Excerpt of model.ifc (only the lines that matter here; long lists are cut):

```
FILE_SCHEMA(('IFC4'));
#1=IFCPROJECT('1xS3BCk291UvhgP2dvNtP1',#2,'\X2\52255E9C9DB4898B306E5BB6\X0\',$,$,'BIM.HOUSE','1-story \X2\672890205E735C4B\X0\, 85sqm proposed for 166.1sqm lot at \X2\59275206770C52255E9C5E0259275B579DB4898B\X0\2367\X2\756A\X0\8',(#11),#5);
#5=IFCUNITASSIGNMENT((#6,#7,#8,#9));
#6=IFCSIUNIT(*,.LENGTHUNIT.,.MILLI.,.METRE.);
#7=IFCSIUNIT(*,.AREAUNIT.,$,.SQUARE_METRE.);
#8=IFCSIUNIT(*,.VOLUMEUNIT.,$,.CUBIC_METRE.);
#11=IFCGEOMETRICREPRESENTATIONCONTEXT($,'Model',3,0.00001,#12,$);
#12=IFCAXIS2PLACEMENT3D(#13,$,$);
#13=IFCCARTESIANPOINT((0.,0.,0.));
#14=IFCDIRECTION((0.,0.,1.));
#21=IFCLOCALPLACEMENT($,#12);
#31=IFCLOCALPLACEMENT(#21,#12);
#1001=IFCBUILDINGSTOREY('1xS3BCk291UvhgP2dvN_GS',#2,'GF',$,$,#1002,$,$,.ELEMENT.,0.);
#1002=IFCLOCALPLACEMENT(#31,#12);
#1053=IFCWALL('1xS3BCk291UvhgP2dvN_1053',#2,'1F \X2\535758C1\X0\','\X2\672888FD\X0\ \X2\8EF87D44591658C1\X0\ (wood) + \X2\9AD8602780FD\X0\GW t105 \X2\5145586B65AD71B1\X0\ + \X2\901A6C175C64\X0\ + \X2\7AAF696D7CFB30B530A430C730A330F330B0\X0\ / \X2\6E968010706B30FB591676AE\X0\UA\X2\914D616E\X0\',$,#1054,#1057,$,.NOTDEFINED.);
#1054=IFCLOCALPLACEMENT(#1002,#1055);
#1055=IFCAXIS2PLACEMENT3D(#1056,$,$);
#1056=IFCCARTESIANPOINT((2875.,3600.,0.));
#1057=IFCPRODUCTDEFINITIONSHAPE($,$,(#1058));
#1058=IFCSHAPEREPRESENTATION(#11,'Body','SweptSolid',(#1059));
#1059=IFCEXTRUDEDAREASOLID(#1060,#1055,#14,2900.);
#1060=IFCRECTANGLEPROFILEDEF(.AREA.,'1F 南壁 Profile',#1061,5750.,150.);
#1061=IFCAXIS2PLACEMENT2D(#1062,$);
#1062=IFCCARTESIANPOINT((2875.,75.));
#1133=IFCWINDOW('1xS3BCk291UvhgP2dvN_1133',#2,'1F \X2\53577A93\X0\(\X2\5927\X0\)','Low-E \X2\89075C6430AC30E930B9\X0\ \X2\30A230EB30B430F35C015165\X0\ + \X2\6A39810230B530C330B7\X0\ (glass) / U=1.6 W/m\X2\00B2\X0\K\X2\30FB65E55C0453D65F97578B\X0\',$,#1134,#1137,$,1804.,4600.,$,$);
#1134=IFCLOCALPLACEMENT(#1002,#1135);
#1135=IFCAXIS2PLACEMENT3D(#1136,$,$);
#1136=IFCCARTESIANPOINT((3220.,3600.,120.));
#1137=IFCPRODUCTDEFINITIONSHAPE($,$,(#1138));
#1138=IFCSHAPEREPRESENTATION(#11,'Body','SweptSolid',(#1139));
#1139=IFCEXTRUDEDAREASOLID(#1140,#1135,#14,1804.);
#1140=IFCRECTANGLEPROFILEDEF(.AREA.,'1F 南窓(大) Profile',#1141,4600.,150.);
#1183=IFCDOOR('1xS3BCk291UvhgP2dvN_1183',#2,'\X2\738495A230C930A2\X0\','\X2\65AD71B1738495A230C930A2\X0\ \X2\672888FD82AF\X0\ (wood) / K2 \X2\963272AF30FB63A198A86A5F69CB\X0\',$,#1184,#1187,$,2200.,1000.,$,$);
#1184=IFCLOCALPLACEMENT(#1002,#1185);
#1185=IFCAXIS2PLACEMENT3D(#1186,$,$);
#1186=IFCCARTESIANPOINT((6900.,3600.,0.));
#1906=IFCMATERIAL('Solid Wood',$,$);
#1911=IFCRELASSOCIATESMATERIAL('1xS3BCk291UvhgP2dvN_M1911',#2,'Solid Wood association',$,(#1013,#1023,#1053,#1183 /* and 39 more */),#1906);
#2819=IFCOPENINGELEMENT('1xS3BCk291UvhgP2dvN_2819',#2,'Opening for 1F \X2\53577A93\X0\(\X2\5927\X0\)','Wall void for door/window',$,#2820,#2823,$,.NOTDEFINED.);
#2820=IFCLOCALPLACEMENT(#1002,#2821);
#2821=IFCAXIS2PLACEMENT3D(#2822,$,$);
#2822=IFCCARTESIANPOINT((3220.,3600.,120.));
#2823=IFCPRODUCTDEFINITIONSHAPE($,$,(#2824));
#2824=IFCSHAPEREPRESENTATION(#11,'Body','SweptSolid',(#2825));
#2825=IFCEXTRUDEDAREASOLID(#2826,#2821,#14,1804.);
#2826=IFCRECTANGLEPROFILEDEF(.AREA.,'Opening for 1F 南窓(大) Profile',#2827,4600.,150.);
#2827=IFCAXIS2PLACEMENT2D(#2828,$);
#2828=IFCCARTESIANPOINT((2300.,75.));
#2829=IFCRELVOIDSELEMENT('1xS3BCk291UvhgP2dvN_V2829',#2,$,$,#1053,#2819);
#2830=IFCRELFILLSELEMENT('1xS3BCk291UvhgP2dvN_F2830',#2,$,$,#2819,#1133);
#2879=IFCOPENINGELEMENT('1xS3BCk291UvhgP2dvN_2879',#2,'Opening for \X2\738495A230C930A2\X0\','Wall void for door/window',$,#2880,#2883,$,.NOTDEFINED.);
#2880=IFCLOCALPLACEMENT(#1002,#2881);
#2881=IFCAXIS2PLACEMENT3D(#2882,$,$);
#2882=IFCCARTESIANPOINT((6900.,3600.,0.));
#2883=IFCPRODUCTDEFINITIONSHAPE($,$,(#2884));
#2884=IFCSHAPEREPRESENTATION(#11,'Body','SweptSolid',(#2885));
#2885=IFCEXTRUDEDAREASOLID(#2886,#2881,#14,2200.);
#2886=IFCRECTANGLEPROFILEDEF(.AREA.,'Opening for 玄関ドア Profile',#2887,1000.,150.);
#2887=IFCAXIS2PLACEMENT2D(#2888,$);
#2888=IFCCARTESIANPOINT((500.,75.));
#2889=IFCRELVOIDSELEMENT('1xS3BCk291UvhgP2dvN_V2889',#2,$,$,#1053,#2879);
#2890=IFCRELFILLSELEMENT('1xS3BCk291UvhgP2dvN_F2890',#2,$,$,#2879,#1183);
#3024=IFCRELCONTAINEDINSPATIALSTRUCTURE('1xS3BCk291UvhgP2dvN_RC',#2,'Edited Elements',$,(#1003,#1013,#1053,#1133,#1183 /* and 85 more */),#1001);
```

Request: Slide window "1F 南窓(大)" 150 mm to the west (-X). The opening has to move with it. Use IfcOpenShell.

```python
import ifcopenshell
import ifcopenshell.api.geometry
import ifcopenshell.util.placement
import ifcopenshell.util.unit

model = ifcopenshell.open("model.ifc")
unit_scale = ifcopenshell.util.unit.calculate_unit_scale(model)

window = model.by_id(1133)
opening = window.FillsVoids[0].RelatingOpeningElement
wall = opening.VoidsElements[0].RelatingBuildingElement

wall_matrix = ifcopenshell.util.placement.get_local_placement(wall.ObjectPlacement)
shift = wall_matrix[:3, 0] * -0.15 / unit_scale
before = ifcopenshell.util.placement.get_local_placement(window.ObjectPlacement)[:3, 3].copy()

# The window is not placed relative to its opening, so move both.
for product in (opening, window):
    matrix = ifcopenshell.util.placement.get_local_placement(product.ObjectPlacement)
    matrix[:3, 3] += shift
    ifcopenshell.api.geometry.edit_object_placement(model, product=product, matrix=matrix, is_si=False)

after = ifcopenshell.util.placement.get_local_placement(window.ObjectPlacement)[:3, 3]
print("window moved by", (after - before).round(3) + 0.0)

model.write("model-out.ifc")
```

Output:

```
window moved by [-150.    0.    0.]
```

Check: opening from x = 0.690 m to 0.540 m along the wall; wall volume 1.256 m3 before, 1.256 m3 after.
